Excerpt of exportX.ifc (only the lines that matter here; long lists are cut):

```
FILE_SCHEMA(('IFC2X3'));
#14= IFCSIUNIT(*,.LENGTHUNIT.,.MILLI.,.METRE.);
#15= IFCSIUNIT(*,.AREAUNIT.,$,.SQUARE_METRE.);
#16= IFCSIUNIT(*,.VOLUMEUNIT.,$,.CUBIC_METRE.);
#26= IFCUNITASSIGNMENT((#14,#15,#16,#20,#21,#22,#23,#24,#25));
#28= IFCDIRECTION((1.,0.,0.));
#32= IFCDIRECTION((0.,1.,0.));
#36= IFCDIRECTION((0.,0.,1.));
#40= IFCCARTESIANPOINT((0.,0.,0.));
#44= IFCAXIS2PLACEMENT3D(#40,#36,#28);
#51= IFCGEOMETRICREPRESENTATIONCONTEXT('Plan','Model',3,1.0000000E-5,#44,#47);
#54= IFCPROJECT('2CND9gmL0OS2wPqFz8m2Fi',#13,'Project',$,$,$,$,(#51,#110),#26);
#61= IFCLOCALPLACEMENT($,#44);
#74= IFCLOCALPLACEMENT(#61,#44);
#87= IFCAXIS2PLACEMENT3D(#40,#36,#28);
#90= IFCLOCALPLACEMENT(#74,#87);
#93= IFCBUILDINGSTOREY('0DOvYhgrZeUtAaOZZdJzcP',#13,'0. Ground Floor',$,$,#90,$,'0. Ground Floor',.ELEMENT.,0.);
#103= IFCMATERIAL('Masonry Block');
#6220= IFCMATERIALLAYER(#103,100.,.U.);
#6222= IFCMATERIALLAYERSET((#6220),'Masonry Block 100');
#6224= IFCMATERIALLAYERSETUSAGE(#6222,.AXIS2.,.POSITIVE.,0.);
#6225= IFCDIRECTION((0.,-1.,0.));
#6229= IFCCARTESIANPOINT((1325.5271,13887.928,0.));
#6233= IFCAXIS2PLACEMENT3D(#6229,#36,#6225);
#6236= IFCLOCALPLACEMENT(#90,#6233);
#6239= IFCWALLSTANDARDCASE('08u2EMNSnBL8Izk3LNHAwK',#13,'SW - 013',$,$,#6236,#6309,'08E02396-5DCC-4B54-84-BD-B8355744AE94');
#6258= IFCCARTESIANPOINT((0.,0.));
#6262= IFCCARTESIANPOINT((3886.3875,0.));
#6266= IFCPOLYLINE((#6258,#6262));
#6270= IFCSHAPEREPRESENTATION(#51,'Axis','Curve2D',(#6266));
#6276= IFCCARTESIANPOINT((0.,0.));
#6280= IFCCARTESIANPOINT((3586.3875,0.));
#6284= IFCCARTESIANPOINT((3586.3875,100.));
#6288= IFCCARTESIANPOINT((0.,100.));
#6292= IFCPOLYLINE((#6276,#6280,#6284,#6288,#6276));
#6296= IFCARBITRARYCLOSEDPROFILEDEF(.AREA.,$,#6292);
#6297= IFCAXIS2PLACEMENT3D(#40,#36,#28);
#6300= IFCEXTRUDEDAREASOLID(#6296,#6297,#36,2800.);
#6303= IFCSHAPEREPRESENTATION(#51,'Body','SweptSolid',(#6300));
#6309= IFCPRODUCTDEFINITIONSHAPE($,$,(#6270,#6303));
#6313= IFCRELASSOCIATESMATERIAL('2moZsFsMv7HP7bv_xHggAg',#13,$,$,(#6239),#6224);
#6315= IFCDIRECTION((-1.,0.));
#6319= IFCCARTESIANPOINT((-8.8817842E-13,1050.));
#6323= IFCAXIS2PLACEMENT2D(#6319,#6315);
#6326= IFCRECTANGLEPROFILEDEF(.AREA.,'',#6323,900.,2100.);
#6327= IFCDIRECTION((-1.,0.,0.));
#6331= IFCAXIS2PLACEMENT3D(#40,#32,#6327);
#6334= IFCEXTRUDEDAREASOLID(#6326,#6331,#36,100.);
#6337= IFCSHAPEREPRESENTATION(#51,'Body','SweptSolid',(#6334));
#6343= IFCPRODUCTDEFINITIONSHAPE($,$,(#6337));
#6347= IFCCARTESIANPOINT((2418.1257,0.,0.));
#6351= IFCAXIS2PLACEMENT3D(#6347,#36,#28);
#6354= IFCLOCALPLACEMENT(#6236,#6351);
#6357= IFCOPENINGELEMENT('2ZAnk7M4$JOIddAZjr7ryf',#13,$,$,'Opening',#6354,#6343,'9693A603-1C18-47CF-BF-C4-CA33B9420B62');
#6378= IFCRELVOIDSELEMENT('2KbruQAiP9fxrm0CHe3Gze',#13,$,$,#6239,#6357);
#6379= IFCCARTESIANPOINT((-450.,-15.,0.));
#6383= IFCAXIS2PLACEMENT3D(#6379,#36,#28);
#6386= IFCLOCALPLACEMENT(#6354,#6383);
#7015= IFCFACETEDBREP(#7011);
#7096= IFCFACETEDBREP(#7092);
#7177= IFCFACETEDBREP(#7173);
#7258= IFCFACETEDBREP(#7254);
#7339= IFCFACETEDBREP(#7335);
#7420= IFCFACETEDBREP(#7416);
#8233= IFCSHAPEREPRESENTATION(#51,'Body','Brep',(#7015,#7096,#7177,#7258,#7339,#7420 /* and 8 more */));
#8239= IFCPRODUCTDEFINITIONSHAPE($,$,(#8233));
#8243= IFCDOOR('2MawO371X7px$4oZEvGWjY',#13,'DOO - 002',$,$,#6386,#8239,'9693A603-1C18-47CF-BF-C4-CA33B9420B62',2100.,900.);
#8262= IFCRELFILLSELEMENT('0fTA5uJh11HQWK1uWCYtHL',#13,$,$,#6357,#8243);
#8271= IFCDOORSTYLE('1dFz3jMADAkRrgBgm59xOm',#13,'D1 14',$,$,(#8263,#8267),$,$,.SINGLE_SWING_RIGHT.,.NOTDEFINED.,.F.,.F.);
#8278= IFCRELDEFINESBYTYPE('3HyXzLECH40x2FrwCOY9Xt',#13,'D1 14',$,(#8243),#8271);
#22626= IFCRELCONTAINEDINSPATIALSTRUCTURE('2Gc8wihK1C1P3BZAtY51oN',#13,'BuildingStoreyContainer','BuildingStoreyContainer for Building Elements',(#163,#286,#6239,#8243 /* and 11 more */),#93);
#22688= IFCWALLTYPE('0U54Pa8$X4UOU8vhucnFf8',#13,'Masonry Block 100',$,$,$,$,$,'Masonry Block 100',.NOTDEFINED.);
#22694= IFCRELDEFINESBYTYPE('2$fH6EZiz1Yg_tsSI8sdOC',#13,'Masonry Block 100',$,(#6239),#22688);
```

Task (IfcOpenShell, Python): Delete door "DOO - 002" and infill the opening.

```python
import ifcopenshell
import ifcopenshell.api.feature
import ifcopenshell.api.root
import ifcopenshell.geom
import ifcopenshell.util.shape

model = ifcopenshell.open("exportX.ifc")
settings = ifcopenshell.geom.settings()


def volume(element):
    """Net volume in cubic metres, openings subtracted."""
    shape = ifcopenshell.geom.create_shape(settings, element)
    return ifcopenshell.util.shape.get_volume(shape.geometry)


door = model.by_id(8243)
opening = door.FillsVoids[0].RelatingOpeningElement
wall = opening.VoidsElements[0].RelatingBuildingElement
before = volume(wall)

ifcopenshell.api.root.remove_product(model, product=door)
ifcopenshell.api.feature.remove_feature(model, feature=opening)

after = volume(wall)

print(f"wall volume {before:.3f} -> {after:.3f} m3")

model.write("exportX_updated.ifc")
```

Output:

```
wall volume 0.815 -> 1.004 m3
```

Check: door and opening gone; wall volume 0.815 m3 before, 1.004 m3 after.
